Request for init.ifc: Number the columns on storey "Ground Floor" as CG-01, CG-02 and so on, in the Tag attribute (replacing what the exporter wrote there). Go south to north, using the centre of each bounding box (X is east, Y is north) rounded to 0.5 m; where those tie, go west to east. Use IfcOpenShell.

First a look at what the model holds.

```python
import ifcopenshell
import ifcopenshell.util.element
import ifcopenshell.util.placement

model = ifcopenshell.open("init.ifc")
print(model.schema)
storey = next(s for s in model.by_type("IfcBuildingStorey") if s.Name == "Ground Floor")
columns = [e for e in ifcopenshell.util.element.get_decomposition(storey) if e.is_a("IfcColumn")]
for e in sorted(columns, key=lambda e: e.id()):
    origin = ifcopenshell.util.placement.get_local_placement(e.ObjectPlacement)[:3, 3]
    print(e.id(), e.Tag, e.Name, origin.round(2) + 0.0, sep=" | ")
```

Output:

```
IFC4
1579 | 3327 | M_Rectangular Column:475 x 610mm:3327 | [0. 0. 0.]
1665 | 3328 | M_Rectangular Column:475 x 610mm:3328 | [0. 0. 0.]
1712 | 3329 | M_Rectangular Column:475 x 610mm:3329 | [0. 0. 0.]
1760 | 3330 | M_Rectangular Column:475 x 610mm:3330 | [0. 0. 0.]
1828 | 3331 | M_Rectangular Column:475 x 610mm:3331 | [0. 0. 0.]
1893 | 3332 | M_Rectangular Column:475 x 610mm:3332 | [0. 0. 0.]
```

```python
import ifcopenshell
import ifcopenshell.geom
import ifcopenshell.util.element
import ifcopenshell.util.shape

model = ifcopenshell.open("init.ifc")
settings = ifcopenshell.geom.settings()
settings.set("use-world-coords", True)


def centre(element):
    shape = ifcopenshell.geom.create_shape(settings, element)
    return ifcopenshell.util.shape.get_bbox_centroid(shape.geometry)


storey = next(s for s in model.by_type("IfcBuildingStorey") if s.Name == "Ground Floor")
columns = [e for e in ifcopenshell.util.element.get_decomposition(storey) if e.is_a("IfcColumn")]

# Insertion points can sit at a corner or the storey origin, so sort by the geometry (in metres).
centres = {e: centre(e) for e in columns}
columns.sort(key=lambda e: (round(centres[e][1] / 0.5), centres[e][0]))

for i, e in enumerate(columns, start=1):
    number = f"CG-{i:02d}"
    e.Tag = number
    print(e.id(), number)

model.write("init_rev.ifc")
```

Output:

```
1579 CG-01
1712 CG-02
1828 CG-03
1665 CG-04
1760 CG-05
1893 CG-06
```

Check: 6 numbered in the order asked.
